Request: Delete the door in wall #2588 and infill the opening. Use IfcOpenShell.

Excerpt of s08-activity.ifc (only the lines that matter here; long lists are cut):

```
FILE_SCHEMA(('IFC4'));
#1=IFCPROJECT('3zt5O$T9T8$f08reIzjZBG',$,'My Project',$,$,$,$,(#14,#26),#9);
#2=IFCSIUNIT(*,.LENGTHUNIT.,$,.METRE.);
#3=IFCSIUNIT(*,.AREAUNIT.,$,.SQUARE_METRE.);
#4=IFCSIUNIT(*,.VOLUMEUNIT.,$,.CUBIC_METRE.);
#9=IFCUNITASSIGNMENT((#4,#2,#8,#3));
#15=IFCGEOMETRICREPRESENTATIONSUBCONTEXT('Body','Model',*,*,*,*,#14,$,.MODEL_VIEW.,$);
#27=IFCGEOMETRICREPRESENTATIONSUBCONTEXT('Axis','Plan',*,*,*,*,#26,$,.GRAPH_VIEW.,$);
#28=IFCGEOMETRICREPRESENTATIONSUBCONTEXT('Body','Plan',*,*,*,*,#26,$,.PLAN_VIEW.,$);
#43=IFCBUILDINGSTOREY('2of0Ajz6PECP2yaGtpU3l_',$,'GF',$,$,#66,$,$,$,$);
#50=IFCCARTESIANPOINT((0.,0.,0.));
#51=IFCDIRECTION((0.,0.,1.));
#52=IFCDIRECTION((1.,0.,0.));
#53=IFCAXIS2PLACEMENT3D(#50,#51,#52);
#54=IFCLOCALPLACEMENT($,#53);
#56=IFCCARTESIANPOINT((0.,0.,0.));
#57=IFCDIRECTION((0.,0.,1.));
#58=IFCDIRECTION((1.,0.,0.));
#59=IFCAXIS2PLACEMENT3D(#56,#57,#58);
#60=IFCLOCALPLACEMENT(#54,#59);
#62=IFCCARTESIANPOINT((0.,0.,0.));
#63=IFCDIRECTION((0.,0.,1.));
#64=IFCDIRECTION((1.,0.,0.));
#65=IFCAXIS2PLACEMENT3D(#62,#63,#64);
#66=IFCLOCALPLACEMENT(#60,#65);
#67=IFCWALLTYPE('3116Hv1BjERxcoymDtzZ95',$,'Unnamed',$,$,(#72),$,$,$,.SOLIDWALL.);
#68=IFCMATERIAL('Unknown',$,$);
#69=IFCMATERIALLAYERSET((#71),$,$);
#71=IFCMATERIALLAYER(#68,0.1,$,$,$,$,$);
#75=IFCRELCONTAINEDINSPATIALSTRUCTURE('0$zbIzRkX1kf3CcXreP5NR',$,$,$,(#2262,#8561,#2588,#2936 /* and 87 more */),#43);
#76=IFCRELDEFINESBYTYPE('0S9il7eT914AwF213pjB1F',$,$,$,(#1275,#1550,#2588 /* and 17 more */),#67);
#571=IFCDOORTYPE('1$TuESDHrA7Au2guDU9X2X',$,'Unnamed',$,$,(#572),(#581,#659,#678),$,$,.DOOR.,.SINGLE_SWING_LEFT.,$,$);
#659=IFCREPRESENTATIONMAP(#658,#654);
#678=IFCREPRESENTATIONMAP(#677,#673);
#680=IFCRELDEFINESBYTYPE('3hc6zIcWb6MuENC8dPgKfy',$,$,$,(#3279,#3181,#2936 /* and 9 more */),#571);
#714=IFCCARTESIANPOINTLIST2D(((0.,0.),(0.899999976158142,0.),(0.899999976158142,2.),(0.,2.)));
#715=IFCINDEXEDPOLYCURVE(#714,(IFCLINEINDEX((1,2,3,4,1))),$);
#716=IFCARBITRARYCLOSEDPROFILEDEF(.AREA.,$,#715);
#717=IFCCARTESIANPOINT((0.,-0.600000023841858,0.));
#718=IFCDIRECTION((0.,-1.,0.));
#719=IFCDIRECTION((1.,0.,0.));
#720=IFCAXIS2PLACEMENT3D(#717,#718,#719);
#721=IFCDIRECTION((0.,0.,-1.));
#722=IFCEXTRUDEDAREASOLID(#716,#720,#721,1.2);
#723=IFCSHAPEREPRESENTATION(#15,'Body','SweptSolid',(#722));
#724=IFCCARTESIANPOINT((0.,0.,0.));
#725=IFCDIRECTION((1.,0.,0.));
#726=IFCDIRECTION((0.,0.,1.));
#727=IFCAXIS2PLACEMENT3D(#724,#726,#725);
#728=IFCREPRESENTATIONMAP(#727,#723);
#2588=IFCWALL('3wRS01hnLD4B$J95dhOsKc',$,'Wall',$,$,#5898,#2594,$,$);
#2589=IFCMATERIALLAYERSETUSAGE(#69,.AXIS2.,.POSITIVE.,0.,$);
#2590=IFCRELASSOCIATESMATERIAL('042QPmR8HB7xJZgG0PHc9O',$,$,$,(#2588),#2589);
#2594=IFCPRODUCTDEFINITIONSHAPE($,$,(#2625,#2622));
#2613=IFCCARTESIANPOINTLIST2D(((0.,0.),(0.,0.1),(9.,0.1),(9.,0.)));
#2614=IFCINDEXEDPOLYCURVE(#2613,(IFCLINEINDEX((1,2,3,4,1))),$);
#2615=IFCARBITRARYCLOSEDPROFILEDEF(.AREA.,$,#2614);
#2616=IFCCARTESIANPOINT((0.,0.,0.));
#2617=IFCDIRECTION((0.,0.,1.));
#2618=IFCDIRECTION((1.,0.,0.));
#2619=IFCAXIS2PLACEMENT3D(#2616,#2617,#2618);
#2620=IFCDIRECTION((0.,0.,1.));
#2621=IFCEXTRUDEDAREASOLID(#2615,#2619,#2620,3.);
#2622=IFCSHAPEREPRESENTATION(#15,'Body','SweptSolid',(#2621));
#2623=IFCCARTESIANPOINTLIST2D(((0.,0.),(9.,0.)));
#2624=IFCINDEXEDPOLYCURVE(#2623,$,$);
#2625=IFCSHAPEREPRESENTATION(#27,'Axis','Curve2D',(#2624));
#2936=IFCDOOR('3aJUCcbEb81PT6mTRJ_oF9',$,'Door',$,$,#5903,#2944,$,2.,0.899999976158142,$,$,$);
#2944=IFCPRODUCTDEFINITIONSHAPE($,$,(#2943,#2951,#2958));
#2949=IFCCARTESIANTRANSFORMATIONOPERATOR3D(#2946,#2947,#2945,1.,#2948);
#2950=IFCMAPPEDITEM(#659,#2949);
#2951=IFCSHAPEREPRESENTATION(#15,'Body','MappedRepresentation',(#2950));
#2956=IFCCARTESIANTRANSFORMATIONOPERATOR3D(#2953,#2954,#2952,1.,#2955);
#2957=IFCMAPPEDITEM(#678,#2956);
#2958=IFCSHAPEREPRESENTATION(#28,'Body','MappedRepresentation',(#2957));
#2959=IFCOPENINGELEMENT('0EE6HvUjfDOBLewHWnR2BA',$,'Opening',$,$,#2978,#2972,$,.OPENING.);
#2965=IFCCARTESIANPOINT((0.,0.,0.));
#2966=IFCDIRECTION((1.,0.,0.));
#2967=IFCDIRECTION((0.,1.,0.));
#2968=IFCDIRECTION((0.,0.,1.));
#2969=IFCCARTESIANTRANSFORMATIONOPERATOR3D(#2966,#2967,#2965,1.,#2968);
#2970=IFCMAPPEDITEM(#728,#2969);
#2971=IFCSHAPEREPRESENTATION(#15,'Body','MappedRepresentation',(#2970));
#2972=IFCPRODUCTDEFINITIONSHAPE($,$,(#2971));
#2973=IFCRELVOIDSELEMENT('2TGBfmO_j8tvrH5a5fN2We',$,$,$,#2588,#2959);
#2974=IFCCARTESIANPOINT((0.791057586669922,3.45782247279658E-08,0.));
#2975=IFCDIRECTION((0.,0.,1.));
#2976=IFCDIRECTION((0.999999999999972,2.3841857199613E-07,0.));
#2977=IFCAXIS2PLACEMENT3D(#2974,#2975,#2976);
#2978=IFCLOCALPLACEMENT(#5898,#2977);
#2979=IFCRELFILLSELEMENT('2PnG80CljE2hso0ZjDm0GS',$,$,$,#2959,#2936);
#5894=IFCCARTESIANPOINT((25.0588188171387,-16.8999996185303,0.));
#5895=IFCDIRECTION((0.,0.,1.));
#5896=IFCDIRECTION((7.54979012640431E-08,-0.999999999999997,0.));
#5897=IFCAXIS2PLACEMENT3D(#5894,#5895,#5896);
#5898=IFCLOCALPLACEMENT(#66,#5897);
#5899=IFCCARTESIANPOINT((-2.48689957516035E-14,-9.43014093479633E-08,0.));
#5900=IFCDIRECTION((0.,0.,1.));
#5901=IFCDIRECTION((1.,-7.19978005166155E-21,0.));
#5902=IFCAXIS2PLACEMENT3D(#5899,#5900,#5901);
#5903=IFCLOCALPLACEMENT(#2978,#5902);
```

```python
import ifcopenshell
import ifcopenshell.api.feature
import ifcopenshell.api.root
import ifcopenshell.geom
import ifcopenshell.util.shape

model = ifcopenshell.open("s08-activity.ifc")
settings = ifcopenshell.geom.settings()


def volume(element):
    """Net volume in cubic metres, openings subtracted."""
    shape = ifcopenshell.geom.create_shape(settings, element)
    return ifcopenshell.util.shape.get_volume(shape.geometry)


door = model.by_guid("3aJUCcbEb81PT6mTRJ_oF9")
opening = door.FillsVoids[0].RelatingOpeningElement
wall = opening.VoidsElements[0].RelatingBuildingElement
before = volume(wall)

ifcopenshell.api.root.remove_product(model, product=door)
ifcopenshell.api.feature.remove_feature(model, feature=opening)

after = volume(wall)

print(f"wall volume {before:.3f} -> {after:.3f} m3")

model.write("s08-activity_edited.ifc")
```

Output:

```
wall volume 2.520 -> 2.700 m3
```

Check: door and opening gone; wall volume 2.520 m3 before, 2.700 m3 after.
